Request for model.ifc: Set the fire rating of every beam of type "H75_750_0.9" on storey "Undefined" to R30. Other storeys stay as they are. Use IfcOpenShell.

First a look at what the model holds.

```python
import ifcopenshell
import ifcopenshell.util.element

model = ifcopenshell.open("model.ifc")
print(model.schema)
storey = next(s for s in model.by_type("IfcBuildingStorey") if s.Name == "Undefined")
beams = [e for e in ifcopenshell.util.element.get_decomposition(storey) if e.is_a("IfcBeam")]
seen = {}
for e in beams:
    element_type = ifcopenshell.util.element.get_type(e)
    key = (element_type.Name if element_type != e and element_type else None, ifcopenshell.util.element.get_pset(e, "Pset_BeamCommon", "FireRating"))
    seen[key] = seen.get(key, 0) + 1
for (name, value), count in sorted(seen.items(), key=str):
    print(count, "x", name, "|", value)
```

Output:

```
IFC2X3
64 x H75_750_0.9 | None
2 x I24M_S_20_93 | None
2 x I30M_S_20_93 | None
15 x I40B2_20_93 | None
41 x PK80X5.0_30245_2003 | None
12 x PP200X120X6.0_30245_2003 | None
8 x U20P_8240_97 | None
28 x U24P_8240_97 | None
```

```python
import ifcopenshell
import ifcopenshell.api.pset
import ifcopenshell.util.element

model = ifcopenshell.open("model.ifc")

storey = next(s for s in model.by_type("IfcBuildingStorey") if s.Name == "Undefined")
beams = [e for e in ifcopenshell.util.element.get_decomposition(storey) if e.is_a("IfcBeam")]

count = 0
for e in beams:
    element_type = ifcopenshell.util.element.get_type(e)
    if element_type in (None, e) or element_type.Name != "H75_750_0.9":
        continue
    found = ifcopenshell.util.element.get_pset(e, "Pset_BeamCommon", should_inherit=False)
    if found:
        pset = model.by_id(found["id"])
        if len(ifcopenshell.util.element.get_elements_by_pset(pset)) > 1:
            pset = ifcopenshell.api.pset.unshare_pset(model, products=[e], pset=pset)[0]
    else:
        pset = ifcopenshell.api.pset.add_pset(model, product=e, name="Pset_BeamCommon")
    ifcopenshell.api.pset.edit_pset(model, pset=pset, properties={"FireRating": "R30"})
    count += 1

print(count, "beams updated")

model.write("model_updated.ifc")
```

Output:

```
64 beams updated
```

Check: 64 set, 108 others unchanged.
